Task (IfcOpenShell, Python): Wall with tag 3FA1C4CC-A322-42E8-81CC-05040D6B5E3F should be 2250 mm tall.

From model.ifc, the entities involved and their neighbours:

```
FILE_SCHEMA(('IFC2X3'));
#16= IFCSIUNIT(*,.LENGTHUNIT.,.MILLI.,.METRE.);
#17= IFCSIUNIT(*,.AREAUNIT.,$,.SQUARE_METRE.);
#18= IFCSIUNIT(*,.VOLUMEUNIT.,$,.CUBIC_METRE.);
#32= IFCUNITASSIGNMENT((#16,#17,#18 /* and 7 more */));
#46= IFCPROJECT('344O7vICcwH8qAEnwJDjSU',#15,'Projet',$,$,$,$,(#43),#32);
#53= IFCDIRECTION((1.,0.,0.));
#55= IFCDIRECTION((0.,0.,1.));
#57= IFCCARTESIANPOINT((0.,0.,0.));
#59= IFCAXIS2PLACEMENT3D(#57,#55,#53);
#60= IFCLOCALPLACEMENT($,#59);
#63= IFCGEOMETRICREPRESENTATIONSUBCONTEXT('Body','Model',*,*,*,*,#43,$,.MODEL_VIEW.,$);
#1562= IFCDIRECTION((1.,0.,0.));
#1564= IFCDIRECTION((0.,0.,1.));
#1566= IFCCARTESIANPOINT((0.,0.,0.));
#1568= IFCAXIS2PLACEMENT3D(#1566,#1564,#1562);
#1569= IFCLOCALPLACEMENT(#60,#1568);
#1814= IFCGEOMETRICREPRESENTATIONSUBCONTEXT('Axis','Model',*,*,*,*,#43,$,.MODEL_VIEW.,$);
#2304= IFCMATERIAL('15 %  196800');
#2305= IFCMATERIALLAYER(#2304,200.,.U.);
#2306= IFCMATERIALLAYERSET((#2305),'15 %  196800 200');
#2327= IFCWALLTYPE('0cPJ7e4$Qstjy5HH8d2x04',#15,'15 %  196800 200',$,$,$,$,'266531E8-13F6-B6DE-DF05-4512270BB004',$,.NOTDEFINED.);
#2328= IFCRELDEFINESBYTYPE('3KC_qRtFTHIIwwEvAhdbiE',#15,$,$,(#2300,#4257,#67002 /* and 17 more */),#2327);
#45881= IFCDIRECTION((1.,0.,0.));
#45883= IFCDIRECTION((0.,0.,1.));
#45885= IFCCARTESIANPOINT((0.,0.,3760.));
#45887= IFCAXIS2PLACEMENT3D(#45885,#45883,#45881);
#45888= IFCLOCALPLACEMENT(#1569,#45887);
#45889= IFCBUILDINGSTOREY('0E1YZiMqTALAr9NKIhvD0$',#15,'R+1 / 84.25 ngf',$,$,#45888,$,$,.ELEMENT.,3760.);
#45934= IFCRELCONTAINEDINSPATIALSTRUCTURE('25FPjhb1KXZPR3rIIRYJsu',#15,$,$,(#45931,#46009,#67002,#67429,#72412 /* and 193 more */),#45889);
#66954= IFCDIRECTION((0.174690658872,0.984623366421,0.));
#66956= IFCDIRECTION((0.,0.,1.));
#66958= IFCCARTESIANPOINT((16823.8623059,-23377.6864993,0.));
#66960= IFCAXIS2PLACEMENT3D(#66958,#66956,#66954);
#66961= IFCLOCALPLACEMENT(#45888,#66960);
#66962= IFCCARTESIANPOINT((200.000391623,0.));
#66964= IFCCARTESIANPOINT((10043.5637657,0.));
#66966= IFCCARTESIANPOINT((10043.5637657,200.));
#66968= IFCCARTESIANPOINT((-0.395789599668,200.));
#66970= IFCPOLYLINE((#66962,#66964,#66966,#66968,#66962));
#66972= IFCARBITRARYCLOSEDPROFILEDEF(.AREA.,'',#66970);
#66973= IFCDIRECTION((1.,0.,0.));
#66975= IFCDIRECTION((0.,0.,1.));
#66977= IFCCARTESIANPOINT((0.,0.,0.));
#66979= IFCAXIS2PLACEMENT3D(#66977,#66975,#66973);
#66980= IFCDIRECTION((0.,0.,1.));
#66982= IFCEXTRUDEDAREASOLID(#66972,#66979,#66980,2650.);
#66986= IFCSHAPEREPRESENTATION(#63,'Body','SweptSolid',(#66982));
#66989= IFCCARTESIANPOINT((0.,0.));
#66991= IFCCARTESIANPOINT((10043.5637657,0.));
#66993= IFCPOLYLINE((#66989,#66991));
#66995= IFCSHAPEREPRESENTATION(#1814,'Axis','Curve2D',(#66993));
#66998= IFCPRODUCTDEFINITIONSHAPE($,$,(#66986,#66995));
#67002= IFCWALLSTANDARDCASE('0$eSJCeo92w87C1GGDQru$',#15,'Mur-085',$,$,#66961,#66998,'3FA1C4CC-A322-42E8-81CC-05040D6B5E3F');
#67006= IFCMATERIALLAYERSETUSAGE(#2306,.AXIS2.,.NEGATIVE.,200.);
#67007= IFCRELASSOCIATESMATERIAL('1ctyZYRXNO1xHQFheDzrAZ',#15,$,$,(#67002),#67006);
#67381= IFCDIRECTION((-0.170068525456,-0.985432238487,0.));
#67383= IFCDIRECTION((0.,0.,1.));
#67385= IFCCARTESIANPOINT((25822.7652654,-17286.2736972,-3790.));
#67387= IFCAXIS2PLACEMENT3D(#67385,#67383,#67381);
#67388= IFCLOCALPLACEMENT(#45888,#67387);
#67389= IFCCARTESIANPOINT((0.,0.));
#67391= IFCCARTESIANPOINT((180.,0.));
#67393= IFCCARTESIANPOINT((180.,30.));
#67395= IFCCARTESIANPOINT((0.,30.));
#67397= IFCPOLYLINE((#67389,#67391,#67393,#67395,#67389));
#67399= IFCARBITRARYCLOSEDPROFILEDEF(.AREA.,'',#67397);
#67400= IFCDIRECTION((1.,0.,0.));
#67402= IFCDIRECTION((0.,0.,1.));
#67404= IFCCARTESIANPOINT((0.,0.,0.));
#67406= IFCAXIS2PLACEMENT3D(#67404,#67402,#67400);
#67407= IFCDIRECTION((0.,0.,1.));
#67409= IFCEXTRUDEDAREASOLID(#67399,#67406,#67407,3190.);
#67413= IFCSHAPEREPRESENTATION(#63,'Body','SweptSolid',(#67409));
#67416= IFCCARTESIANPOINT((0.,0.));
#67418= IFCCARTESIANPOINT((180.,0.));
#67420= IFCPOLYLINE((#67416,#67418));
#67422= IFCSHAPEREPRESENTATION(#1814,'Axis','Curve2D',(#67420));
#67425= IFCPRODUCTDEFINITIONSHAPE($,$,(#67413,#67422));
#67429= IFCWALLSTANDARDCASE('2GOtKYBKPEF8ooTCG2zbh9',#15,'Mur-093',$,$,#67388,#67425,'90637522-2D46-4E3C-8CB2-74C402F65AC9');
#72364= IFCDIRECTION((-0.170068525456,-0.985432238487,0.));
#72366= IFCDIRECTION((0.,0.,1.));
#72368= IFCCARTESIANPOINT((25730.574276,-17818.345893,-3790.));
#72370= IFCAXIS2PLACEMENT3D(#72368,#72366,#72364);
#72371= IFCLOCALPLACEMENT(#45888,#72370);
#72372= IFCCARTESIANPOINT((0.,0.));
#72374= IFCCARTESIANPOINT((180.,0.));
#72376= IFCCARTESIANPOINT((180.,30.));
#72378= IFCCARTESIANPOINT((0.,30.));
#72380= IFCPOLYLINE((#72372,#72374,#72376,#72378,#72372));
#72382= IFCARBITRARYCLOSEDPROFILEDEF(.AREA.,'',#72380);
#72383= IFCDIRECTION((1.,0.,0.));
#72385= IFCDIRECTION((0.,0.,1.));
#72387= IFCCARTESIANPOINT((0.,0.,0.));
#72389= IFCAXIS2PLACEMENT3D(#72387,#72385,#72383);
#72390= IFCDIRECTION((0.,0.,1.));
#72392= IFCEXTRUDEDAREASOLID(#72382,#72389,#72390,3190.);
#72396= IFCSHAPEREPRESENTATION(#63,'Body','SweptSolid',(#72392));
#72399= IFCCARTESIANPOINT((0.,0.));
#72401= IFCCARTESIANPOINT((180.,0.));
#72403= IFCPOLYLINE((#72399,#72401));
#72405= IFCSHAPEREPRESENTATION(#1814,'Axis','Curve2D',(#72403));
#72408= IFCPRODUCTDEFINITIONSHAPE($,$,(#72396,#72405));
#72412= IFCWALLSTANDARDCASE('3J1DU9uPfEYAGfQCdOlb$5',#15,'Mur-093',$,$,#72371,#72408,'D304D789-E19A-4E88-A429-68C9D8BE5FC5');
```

```python
import ifcopenshell
import ifcopenshell.geom
import ifcopenshell.util.representation
import ifcopenshell.util.shape

model = ifcopenshell.open("model.ifc")
settings = ifcopenshell.geom.settings()


def volume(element):
    """Net volume in cubic metres, openings subtracted."""
    shape = ifcopenshell.geom.create_shape(settings, element)
    return ifcopenshell.util.shape.get_volume(shape.geometry)


wall = model.by_id(67002)
before = volume(wall)

body = ifcopenshell.util.representation.get_representation(wall, "Model", "Body")
solid = body.Items[0]
old_height = solid.Depth
solid.Depth = 2250.0
after = volume(wall)

print(f"height {old_height:g} -> {solid.Depth:g}, volume {before:.3f} -> {after:.3f} m3")

model.write("model_edited.ifc")
```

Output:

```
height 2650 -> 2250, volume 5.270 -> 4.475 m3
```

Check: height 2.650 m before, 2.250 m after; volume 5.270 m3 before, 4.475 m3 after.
